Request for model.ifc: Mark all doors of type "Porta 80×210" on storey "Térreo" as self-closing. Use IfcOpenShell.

First a look at what the model holds.

```python
import ifcopenshell
import ifcopenshell.util.element

model = ifcopenshell.open("model.ifc")
print(model.schema)
storey = next(s for s in model.by_type("IfcBuildingStorey") if s.Name == "Térreo")
doors = [e for e in ifcopenshell.util.element.get_decomposition(storey) if e.is_a("IfcDoor")]
seen = {}
for e in doors:
    element_type = ifcopenshell.util.element.get_type(e)
    key = (element_type.Name if element_type != e and element_type else None, ifcopenshell.util.element.get_pset(e, "Pset_DoorCommon", "SelfClosing"))
    seen[key] = seen.get(key, 0) + 1
for (name, value), count in sorted(seen.items(), key=str):
    print(count, "x", name, "|", value)
```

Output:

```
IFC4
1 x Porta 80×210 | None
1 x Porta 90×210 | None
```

```python
import ifcopenshell
import ifcopenshell.api.pset
import ifcopenshell.util.element

model = ifcopenshell.open("model.ifc")

storey = next(s for s in model.by_type("IfcBuildingStorey") if s.Name == "Térreo")
doors = [e for e in ifcopenshell.util.element.get_decomposition(storey) if e.is_a("IfcDoor")]

count = 0
for e in doors:
    element_type = ifcopenshell.util.element.get_type(e)
    if element_type in (None, e) or element_type.Name != "Porta 80×210":
        continue
    # add_pset returns the element's existing set when there is one.
    pset = ifcopenshell.api.pset.add_pset(model, product=e, name="Pset_DoorCommon")
    ifcopenshell.api.pset.edit_pset(model, pset=pset, properties={"SelfClosing": True})
    count += 1

print(count, "doors updated")

model.write("model_v2.ifc")
```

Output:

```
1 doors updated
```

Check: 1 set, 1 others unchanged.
